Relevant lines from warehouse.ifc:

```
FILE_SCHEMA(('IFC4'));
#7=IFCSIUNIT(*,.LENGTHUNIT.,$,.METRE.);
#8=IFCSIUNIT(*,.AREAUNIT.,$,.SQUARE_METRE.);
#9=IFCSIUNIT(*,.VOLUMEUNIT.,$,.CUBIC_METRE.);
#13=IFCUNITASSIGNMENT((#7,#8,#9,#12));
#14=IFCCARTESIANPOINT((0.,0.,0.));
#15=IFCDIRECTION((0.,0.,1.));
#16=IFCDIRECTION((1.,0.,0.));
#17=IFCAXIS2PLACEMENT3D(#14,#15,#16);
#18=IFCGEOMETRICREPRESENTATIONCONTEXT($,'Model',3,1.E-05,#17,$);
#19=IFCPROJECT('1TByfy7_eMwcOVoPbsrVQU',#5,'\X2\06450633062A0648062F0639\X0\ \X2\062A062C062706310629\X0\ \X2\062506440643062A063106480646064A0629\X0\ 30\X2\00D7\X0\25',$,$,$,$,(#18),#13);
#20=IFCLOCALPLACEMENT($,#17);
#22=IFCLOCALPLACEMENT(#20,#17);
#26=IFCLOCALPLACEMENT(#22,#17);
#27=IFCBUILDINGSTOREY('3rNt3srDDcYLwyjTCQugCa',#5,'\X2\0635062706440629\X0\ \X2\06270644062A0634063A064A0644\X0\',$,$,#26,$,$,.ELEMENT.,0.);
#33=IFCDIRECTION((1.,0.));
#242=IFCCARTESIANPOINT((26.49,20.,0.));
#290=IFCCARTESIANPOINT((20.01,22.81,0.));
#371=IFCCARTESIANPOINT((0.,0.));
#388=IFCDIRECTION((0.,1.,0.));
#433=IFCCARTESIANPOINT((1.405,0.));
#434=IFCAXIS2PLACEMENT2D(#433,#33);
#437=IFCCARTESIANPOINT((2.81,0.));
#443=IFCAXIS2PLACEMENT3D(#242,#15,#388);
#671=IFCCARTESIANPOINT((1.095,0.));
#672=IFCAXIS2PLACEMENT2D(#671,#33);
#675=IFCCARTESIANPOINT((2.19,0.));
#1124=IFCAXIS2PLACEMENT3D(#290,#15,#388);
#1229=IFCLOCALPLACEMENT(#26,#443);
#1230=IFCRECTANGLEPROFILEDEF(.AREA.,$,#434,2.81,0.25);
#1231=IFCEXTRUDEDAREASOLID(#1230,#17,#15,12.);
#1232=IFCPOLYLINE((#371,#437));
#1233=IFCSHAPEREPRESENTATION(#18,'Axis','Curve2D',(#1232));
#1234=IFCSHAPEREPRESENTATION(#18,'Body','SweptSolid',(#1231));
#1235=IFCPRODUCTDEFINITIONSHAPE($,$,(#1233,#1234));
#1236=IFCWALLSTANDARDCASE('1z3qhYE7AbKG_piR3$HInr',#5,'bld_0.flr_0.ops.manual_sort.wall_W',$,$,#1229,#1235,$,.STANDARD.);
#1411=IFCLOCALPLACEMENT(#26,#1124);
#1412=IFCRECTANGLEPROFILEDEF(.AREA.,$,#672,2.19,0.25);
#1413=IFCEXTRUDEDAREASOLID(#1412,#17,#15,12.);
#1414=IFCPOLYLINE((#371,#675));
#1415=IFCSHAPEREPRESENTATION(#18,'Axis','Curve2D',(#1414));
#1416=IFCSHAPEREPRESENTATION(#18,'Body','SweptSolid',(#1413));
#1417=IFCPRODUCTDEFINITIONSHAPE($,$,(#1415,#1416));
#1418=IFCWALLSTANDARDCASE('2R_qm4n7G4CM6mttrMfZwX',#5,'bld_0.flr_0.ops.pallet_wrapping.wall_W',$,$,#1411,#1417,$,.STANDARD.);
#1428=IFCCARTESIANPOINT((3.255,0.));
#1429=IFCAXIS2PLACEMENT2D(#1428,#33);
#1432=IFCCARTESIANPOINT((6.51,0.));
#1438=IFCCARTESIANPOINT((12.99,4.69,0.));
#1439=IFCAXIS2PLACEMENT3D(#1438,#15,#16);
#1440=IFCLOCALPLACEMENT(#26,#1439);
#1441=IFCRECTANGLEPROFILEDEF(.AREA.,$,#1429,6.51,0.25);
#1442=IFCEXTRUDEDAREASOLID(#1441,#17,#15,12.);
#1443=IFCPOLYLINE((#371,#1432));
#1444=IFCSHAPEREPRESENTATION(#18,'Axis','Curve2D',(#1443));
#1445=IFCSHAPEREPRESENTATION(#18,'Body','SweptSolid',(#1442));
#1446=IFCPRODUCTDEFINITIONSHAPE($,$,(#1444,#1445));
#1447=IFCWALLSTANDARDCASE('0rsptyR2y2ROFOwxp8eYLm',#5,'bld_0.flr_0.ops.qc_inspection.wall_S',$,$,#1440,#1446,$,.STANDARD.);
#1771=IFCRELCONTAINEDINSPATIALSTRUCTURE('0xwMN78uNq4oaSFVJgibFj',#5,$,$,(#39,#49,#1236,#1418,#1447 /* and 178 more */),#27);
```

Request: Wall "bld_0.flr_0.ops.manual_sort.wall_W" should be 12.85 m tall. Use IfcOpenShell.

```python
import ifcopenshell
import ifcopenshell.geom
import ifcopenshell.util.shape
import ifcopenshell.util.unit

model = ifcopenshell.open("warehouse.ifc")
unit_scale = ifcopenshell.util.unit.calculate_unit_scale(model)
settings = ifcopenshell.geom.settings()


def volume(element):
    """Net volume in cubic metres, openings subtracted."""
    shape = ifcopenshell.geom.create_shape(settings, element)
    return ifcopenshell.util.shape.get_volume(shape.geometry)


wall = model.by_guid("1z3qhYE7AbKG_piR3$HInr")
before = volume(wall)

body = next(r for r in wall.Representation.Representations if r.RepresentationIdentifier == "Body")
solid = body.Items[0]
old_height = solid.Depth
solid.Depth = 12.85 / unit_scale
after = volume(wall)

print(f"height {old_height:g} -> {solid.Depth:g}, volume {before:.3f} -> {after:.3f} m3")

model.write("warehouse_updated.ifc")
```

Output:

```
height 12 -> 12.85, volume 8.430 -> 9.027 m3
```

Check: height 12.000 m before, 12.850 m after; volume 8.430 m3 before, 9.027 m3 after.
